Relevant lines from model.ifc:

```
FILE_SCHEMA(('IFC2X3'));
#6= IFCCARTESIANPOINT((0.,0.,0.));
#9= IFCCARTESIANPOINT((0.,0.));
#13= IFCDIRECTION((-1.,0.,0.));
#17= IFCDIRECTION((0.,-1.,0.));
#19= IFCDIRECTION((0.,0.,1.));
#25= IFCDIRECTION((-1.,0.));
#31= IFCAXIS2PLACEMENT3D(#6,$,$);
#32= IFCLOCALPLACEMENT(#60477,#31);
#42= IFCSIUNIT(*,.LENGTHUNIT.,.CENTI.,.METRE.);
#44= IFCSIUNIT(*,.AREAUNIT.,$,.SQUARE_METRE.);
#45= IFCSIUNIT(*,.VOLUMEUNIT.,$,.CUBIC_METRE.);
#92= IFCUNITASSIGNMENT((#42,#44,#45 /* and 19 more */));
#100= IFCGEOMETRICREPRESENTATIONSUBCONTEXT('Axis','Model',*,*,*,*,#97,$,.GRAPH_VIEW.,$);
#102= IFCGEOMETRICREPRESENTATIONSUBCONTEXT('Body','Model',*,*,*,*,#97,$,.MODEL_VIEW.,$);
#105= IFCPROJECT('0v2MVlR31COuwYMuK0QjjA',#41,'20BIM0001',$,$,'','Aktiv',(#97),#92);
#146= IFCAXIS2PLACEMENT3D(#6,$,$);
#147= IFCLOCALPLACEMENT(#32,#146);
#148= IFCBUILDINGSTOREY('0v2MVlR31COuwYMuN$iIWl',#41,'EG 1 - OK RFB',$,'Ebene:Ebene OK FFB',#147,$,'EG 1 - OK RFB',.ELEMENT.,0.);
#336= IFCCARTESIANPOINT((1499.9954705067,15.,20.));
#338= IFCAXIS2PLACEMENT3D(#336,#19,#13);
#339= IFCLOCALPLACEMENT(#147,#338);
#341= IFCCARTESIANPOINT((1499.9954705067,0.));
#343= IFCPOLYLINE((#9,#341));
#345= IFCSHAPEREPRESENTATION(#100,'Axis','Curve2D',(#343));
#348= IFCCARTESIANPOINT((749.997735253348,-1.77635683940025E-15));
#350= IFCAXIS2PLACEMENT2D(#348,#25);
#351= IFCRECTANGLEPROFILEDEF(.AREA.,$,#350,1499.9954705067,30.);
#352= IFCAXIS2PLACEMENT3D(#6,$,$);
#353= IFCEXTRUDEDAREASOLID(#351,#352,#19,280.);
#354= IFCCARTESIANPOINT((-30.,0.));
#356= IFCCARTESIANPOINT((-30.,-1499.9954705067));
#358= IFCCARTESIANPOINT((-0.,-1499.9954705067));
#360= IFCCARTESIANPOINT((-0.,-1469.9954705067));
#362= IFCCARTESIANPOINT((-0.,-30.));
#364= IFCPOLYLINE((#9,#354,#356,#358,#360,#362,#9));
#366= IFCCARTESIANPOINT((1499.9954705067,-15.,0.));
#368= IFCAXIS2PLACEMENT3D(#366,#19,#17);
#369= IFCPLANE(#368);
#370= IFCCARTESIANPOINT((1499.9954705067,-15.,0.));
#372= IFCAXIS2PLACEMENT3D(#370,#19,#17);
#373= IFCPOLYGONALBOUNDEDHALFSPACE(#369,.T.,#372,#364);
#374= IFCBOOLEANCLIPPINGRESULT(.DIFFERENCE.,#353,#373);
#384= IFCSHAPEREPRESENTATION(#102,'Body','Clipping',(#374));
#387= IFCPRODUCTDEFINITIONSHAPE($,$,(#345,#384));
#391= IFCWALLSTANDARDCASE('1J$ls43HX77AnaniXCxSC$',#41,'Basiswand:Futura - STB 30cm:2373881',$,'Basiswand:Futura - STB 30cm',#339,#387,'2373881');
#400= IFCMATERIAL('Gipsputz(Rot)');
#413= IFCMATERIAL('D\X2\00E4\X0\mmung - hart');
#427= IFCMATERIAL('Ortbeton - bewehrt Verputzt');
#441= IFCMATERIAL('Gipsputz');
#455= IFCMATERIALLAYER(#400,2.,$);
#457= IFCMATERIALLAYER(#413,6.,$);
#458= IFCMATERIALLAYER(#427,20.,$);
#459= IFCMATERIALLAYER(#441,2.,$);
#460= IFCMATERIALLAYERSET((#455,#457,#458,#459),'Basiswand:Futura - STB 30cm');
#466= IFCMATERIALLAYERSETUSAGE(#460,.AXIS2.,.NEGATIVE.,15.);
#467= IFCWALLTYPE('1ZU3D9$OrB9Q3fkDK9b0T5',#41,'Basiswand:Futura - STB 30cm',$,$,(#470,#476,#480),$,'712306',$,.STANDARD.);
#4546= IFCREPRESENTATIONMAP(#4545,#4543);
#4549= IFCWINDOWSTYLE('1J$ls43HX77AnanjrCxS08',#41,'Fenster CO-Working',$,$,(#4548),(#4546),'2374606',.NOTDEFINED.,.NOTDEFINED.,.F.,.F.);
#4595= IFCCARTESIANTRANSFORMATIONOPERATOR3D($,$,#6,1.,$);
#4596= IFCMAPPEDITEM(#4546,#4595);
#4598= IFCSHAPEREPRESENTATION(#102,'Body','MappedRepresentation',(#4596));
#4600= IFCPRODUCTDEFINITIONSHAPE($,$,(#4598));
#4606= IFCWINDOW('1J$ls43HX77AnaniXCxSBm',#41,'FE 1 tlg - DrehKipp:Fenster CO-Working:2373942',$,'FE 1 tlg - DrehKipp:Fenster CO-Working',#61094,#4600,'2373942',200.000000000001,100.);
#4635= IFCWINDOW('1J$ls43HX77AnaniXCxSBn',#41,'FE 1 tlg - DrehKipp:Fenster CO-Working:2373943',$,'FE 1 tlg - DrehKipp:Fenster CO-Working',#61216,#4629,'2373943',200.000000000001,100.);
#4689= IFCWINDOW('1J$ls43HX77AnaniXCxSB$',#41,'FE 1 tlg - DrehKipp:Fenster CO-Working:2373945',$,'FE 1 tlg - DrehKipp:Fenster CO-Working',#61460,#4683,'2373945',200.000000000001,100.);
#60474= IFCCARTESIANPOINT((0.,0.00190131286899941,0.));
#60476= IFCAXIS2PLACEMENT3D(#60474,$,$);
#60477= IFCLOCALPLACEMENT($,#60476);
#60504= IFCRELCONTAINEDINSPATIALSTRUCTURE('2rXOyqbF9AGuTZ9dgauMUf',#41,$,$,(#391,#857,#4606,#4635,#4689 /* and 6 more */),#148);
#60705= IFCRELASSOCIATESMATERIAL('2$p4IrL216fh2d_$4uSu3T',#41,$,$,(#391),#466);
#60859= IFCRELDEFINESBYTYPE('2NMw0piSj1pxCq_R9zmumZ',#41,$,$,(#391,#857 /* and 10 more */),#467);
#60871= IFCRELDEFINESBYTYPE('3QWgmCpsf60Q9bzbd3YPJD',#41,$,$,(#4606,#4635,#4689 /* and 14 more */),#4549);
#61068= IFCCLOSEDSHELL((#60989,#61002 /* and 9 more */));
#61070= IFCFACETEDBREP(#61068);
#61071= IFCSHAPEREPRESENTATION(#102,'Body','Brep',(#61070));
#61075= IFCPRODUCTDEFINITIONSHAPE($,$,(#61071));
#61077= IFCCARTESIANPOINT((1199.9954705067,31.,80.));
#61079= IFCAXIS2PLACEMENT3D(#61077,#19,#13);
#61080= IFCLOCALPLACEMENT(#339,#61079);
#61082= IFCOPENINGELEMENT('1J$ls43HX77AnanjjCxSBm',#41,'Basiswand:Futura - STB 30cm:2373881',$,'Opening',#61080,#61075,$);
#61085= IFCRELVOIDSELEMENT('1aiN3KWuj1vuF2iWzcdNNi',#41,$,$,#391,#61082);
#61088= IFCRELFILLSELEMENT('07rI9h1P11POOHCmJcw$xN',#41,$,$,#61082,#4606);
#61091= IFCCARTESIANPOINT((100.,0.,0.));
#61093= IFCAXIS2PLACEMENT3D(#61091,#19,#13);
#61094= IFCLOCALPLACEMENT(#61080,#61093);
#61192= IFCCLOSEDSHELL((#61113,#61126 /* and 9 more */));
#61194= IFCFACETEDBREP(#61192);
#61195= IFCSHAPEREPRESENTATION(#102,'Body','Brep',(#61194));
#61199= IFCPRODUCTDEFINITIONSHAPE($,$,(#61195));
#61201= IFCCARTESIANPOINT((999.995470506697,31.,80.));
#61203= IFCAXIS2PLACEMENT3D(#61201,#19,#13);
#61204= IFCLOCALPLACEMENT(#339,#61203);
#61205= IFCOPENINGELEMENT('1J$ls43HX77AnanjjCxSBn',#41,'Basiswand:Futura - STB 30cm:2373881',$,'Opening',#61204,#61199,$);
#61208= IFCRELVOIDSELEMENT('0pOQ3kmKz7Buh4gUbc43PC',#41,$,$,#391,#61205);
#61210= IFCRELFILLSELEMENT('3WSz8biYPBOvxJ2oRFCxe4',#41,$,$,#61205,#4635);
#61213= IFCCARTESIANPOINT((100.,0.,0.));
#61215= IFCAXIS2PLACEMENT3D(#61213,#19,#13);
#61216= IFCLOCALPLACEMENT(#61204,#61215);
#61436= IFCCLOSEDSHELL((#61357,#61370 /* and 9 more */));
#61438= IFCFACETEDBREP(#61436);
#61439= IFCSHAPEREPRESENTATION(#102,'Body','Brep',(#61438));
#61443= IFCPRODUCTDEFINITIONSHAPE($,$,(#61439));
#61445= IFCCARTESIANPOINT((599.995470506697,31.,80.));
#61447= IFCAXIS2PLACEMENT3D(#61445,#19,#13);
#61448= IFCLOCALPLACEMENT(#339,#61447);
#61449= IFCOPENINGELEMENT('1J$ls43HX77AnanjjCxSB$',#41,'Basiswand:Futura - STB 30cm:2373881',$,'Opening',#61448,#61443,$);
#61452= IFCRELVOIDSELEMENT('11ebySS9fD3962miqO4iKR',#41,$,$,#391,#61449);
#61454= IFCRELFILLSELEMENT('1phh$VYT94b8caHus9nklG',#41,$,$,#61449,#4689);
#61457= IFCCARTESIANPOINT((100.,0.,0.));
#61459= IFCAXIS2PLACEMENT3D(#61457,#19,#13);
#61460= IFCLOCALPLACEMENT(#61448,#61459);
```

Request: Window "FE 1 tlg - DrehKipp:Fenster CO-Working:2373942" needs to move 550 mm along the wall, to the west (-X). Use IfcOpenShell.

```python
import ifcopenshell
import ifcopenshell.api.geometry
import ifcopenshell.util.placement
import ifcopenshell.util.unit

model = ifcopenshell.open("model.ifc")
unit_scale = ifcopenshell.util.unit.calculate_unit_scale(model)

window = model.by_id(4606)
opening = window.FillsVoids[0].RelatingOpeningElement
wall = opening.VoidsElements[0].RelatingBuildingElement

wall_matrix = ifcopenshell.util.placement.get_local_placement(wall.ObjectPlacement)
shift = wall_matrix[:3, 0] * 0.55 / unit_scale
before = ifcopenshell.util.placement.get_local_placement(window.ObjectPlacement)[:3, 3].copy()

# The window is placed relative to its opening, so it follows when the opening moves.
matrix = ifcopenshell.util.placement.get_local_placement(opening.ObjectPlacement)
matrix[:3, 3] += shift
ifcopenshell.api.geometry.edit_object_placement(
    model, product=opening, matrix=matrix, is_si=False, should_transform_children=True
)

after = ifcopenshell.util.placement.get_local_placement(window.ObjectPlacement)[:3, 3]
print("window moved by", (after - before).round(3) + 0.0)

model.write("model_v2.ifc")
```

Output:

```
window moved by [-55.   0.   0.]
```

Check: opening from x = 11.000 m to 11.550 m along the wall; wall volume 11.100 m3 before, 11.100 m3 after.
